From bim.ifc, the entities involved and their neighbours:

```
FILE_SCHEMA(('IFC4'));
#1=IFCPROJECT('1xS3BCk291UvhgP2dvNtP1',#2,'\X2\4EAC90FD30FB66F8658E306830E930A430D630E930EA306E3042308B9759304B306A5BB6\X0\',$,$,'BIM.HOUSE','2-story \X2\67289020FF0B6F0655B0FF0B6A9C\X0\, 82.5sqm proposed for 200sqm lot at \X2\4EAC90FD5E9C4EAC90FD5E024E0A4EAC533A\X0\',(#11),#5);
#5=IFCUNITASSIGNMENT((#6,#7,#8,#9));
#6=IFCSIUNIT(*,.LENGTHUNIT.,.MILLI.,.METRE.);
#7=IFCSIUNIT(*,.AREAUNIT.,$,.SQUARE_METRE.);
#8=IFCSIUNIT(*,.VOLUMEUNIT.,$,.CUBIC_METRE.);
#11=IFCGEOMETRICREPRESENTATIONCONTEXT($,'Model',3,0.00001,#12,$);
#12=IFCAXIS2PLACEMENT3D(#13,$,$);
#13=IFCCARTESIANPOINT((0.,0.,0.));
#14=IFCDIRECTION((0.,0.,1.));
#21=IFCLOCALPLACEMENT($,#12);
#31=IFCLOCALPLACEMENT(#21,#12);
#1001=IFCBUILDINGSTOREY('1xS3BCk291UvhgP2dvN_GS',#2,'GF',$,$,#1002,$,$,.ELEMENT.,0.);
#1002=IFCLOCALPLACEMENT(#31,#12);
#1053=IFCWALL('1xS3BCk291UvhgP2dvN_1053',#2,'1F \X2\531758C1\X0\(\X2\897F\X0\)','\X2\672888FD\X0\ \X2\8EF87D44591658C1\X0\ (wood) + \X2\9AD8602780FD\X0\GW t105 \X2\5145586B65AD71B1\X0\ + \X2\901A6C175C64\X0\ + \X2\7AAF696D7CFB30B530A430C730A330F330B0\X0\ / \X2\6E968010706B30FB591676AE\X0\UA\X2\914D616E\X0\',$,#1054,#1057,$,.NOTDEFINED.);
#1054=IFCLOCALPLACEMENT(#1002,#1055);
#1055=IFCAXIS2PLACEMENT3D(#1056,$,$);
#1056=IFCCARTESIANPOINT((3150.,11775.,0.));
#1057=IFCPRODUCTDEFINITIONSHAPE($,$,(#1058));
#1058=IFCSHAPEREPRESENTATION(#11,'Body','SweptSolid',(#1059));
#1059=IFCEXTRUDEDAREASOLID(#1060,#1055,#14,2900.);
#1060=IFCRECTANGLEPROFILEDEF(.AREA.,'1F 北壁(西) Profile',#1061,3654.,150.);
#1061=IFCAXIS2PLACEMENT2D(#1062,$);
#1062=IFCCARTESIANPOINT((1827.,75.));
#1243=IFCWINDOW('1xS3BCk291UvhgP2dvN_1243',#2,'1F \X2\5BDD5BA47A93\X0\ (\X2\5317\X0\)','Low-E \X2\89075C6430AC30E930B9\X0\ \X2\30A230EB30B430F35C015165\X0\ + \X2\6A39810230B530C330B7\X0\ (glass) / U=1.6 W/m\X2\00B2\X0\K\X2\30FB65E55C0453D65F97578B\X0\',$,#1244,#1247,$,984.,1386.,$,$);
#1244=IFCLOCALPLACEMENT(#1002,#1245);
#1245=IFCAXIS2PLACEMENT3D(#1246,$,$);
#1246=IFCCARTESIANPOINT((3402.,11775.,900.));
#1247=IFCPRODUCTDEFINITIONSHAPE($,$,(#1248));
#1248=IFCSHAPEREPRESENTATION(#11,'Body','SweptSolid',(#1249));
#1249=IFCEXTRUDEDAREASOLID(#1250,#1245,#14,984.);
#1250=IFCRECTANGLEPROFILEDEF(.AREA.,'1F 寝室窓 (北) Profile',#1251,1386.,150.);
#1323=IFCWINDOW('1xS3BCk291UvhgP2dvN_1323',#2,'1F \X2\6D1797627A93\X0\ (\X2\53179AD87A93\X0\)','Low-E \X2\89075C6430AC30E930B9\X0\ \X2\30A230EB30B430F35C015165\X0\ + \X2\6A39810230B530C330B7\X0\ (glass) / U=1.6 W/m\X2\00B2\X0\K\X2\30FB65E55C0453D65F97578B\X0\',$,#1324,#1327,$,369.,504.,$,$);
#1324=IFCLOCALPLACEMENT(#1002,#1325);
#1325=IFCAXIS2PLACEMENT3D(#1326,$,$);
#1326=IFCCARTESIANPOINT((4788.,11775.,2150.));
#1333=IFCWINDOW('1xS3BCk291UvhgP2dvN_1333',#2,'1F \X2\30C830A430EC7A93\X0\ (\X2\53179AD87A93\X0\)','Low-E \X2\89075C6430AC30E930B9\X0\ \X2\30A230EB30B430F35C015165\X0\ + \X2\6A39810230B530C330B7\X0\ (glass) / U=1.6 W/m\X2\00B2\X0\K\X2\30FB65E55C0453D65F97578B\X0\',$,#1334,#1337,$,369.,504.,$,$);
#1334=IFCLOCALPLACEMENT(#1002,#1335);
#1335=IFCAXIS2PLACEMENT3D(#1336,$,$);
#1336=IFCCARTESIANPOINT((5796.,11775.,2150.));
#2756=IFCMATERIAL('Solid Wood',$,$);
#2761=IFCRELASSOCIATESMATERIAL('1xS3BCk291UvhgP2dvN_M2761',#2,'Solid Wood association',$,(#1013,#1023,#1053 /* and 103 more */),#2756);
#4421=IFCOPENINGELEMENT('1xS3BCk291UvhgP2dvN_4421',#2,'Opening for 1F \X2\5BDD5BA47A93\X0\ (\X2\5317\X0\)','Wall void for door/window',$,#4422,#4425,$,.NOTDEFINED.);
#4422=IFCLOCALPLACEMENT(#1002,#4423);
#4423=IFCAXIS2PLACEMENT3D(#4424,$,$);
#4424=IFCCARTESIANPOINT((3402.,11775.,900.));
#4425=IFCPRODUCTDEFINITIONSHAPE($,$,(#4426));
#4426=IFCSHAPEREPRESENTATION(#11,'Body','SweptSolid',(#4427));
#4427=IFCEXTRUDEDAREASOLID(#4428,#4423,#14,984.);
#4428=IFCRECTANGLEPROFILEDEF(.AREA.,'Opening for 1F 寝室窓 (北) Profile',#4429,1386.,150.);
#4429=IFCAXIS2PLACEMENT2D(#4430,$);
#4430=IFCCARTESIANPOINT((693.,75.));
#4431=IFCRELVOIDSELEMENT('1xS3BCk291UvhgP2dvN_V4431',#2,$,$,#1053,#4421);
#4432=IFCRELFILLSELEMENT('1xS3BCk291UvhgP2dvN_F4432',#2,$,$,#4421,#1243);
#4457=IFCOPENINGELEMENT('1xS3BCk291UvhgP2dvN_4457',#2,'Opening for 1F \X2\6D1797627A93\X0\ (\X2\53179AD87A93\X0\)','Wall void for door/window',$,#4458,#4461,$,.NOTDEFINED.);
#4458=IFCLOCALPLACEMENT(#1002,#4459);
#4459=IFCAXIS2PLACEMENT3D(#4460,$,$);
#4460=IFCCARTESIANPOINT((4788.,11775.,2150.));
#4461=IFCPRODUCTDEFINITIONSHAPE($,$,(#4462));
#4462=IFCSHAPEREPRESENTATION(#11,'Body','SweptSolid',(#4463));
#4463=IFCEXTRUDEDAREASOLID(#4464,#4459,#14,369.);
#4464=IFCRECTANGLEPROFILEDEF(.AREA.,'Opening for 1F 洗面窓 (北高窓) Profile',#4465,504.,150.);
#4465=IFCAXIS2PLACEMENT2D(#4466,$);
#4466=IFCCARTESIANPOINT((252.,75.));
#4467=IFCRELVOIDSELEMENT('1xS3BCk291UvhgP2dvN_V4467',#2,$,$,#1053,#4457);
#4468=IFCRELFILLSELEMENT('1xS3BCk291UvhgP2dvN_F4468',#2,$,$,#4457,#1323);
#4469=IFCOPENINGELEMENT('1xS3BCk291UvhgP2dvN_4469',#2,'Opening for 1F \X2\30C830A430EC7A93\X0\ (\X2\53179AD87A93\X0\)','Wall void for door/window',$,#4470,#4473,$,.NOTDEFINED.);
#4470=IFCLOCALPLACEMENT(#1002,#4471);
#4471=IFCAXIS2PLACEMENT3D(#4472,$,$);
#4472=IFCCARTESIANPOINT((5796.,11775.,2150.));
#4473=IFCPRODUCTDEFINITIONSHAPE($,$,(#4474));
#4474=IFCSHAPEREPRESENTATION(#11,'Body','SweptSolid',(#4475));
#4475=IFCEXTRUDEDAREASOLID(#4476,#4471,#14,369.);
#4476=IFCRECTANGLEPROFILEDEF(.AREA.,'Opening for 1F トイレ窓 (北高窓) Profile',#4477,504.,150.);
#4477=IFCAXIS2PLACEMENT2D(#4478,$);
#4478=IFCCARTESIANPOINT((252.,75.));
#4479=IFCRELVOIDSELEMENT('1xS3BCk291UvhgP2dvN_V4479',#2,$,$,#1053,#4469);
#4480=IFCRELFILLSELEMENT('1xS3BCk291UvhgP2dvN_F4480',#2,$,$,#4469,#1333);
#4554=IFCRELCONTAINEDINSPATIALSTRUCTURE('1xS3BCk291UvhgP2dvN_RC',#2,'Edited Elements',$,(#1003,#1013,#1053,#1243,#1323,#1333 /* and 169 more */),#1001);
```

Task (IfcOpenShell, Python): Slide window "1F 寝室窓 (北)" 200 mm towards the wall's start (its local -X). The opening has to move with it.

```python
import ifcopenshell
import ifcopenshell.api.geometry
import ifcopenshell.util.placement

model = ifcopenshell.open("bim.ifc")

window = model.by_id(1243)
opening = window.FillsVoids[0].RelatingOpeningElement
wall = opening.VoidsElements[0].RelatingBuildingElement

wall_matrix = ifcopenshell.util.placement.get_local_placement(wall.ObjectPlacement)
shift = wall_matrix[:3, 0] * -200.0
before = ifcopenshell.util.placement.get_local_placement(window.ObjectPlacement)[:3, 3].copy()

# The window is not placed relative to its opening, so move both.
for product in (opening, window):
    matrix = ifcopenshell.util.placement.get_local_placement(product.ObjectPlacement)
    matrix[:3, 3] += shift
    ifcopenshell.api.geometry.edit_object_placement(model, product=product, matrix=matrix, is_si=False)

after = ifcopenshell.util.placement.get_local_placement(window.ObjectPlacement)[:3, 3]
print("window moved by", (after - before).round(3) + 0.0)

model.write("bim-out.ifc")
```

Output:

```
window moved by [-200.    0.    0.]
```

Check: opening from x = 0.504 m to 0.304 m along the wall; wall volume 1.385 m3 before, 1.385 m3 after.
